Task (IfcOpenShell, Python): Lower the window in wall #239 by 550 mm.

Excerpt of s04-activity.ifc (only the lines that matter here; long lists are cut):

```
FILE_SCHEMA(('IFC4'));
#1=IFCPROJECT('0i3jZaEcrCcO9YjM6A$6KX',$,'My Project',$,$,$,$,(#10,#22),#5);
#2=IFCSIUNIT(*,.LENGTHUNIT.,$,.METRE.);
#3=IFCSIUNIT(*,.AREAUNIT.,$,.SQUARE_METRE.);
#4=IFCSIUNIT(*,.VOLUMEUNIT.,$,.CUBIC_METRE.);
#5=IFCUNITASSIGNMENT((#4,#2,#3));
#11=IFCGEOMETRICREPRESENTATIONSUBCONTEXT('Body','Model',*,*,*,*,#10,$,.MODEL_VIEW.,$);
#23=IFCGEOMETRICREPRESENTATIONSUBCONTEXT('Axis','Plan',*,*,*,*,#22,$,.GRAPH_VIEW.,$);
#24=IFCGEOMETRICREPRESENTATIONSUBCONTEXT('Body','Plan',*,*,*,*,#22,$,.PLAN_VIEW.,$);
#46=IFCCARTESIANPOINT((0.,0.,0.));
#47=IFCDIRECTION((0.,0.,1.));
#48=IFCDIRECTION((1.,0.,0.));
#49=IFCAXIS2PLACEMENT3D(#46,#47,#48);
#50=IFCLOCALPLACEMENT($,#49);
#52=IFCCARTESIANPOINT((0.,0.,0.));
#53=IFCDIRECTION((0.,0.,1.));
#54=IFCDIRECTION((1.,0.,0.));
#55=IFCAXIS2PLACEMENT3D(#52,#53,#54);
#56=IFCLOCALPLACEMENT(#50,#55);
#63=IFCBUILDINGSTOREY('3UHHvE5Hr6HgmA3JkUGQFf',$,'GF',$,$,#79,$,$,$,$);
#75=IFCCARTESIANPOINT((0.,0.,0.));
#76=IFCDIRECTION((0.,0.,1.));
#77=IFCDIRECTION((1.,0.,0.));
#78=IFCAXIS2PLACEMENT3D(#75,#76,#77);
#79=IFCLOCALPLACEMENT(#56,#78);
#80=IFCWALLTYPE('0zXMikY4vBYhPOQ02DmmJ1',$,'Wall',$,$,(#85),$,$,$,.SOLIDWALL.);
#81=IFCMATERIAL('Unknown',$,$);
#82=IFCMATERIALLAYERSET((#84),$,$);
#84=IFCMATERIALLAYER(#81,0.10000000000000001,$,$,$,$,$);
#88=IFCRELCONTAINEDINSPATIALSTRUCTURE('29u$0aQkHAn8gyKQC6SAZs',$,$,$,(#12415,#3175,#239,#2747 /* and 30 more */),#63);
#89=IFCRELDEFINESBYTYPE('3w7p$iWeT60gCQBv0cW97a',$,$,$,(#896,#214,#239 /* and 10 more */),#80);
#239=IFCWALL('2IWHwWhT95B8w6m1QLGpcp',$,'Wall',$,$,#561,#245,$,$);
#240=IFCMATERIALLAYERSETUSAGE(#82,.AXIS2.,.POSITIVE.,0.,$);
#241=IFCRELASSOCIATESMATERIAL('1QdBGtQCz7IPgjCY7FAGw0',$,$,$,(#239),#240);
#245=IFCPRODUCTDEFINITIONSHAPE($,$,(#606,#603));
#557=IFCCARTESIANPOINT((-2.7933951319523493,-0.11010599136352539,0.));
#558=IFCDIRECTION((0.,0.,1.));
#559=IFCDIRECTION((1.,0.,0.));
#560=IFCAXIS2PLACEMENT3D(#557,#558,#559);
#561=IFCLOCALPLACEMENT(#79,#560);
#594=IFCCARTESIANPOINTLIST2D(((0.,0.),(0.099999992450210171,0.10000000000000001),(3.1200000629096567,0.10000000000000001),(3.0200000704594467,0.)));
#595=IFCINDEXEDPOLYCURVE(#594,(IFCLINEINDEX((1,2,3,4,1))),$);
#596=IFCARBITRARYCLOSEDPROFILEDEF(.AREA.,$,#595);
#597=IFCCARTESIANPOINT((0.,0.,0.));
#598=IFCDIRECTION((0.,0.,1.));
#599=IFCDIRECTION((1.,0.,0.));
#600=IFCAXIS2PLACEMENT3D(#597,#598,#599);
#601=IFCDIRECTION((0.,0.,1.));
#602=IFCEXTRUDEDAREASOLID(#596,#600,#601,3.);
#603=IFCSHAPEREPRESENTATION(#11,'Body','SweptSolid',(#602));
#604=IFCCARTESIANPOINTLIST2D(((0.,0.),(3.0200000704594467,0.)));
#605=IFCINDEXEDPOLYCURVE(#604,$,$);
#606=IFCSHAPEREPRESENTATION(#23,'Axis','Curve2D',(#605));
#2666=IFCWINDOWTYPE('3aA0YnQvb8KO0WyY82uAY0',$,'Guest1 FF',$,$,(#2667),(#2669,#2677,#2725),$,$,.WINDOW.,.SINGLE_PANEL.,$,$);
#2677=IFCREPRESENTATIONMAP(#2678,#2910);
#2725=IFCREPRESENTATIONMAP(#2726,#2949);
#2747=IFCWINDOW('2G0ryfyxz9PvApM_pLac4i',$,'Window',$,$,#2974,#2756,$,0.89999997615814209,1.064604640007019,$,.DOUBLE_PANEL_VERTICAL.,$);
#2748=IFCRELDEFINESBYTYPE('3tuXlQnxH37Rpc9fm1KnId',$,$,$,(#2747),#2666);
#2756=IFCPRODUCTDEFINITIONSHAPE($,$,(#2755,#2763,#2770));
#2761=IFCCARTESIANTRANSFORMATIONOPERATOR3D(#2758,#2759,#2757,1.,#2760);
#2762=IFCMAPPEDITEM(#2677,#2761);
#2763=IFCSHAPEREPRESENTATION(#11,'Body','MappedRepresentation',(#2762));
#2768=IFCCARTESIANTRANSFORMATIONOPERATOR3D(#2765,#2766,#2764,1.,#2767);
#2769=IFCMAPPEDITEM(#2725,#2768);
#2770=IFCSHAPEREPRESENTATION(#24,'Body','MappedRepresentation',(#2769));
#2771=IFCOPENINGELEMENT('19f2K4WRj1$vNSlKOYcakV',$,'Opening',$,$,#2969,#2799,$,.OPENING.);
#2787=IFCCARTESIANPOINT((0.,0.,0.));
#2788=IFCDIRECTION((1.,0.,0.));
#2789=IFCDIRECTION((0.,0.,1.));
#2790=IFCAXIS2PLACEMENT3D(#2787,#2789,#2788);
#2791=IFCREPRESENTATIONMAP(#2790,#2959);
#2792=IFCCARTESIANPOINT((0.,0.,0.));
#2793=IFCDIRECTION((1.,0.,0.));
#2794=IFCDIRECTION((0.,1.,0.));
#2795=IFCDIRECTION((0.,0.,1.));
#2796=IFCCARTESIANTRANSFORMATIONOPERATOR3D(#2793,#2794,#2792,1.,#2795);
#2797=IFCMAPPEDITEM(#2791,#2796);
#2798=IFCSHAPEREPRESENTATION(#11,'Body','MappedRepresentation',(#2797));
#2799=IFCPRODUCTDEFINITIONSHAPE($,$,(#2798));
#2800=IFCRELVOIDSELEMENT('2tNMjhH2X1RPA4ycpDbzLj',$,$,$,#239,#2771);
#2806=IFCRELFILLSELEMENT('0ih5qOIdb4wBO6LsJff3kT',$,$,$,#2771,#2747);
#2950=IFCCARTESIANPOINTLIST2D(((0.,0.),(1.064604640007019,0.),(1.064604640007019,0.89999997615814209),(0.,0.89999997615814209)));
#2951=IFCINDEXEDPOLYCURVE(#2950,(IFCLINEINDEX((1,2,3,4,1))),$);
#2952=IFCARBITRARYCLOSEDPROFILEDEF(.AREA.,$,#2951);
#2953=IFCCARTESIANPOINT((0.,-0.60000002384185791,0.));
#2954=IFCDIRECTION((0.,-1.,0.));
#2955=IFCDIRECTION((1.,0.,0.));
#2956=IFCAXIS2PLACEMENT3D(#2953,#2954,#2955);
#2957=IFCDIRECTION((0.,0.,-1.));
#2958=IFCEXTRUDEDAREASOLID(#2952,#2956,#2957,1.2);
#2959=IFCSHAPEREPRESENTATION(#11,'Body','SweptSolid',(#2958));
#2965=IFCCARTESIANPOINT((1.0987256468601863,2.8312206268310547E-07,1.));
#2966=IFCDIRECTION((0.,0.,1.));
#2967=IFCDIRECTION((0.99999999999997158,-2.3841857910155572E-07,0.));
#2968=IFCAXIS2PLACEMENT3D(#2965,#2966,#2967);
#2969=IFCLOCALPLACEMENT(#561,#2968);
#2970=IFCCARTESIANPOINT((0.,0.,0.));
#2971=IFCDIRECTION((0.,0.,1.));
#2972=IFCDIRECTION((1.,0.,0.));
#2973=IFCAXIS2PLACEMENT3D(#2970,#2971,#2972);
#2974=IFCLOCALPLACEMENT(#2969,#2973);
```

```python
import numpy as np
import ifcopenshell
import ifcopenshell.api.geometry
import ifcopenshell.util.placement
import ifcopenshell.util.unit

model = ifcopenshell.open("s04-activity.ifc")
unit_scale = ifcopenshell.util.unit.calculate_unit_scale(model)

window = model.by_guid("2G0ryfyxz9PvApM_pLac4i")
opening = window.FillsVoids[0].RelatingOpeningElement
dz = -0.55 / unit_scale

shift = np.array([0.0, 0.0, dz])
# The window is placed relative to its opening, so it follows when the opening moves.
matrix = ifcopenshell.util.placement.get_local_placement(opening.ObjectPlacement)
matrix[:3, 3] += shift
ifcopenshell.api.geometry.edit_object_placement(
    model, product=opening, matrix=matrix, is_si=False, should_transform_children=True
)

print(f"moved by {dz * unit_scale:+.3f} m")

model.write("s04-activity-out.ifc")
```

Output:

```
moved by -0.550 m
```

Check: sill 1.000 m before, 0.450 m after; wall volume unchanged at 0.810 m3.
